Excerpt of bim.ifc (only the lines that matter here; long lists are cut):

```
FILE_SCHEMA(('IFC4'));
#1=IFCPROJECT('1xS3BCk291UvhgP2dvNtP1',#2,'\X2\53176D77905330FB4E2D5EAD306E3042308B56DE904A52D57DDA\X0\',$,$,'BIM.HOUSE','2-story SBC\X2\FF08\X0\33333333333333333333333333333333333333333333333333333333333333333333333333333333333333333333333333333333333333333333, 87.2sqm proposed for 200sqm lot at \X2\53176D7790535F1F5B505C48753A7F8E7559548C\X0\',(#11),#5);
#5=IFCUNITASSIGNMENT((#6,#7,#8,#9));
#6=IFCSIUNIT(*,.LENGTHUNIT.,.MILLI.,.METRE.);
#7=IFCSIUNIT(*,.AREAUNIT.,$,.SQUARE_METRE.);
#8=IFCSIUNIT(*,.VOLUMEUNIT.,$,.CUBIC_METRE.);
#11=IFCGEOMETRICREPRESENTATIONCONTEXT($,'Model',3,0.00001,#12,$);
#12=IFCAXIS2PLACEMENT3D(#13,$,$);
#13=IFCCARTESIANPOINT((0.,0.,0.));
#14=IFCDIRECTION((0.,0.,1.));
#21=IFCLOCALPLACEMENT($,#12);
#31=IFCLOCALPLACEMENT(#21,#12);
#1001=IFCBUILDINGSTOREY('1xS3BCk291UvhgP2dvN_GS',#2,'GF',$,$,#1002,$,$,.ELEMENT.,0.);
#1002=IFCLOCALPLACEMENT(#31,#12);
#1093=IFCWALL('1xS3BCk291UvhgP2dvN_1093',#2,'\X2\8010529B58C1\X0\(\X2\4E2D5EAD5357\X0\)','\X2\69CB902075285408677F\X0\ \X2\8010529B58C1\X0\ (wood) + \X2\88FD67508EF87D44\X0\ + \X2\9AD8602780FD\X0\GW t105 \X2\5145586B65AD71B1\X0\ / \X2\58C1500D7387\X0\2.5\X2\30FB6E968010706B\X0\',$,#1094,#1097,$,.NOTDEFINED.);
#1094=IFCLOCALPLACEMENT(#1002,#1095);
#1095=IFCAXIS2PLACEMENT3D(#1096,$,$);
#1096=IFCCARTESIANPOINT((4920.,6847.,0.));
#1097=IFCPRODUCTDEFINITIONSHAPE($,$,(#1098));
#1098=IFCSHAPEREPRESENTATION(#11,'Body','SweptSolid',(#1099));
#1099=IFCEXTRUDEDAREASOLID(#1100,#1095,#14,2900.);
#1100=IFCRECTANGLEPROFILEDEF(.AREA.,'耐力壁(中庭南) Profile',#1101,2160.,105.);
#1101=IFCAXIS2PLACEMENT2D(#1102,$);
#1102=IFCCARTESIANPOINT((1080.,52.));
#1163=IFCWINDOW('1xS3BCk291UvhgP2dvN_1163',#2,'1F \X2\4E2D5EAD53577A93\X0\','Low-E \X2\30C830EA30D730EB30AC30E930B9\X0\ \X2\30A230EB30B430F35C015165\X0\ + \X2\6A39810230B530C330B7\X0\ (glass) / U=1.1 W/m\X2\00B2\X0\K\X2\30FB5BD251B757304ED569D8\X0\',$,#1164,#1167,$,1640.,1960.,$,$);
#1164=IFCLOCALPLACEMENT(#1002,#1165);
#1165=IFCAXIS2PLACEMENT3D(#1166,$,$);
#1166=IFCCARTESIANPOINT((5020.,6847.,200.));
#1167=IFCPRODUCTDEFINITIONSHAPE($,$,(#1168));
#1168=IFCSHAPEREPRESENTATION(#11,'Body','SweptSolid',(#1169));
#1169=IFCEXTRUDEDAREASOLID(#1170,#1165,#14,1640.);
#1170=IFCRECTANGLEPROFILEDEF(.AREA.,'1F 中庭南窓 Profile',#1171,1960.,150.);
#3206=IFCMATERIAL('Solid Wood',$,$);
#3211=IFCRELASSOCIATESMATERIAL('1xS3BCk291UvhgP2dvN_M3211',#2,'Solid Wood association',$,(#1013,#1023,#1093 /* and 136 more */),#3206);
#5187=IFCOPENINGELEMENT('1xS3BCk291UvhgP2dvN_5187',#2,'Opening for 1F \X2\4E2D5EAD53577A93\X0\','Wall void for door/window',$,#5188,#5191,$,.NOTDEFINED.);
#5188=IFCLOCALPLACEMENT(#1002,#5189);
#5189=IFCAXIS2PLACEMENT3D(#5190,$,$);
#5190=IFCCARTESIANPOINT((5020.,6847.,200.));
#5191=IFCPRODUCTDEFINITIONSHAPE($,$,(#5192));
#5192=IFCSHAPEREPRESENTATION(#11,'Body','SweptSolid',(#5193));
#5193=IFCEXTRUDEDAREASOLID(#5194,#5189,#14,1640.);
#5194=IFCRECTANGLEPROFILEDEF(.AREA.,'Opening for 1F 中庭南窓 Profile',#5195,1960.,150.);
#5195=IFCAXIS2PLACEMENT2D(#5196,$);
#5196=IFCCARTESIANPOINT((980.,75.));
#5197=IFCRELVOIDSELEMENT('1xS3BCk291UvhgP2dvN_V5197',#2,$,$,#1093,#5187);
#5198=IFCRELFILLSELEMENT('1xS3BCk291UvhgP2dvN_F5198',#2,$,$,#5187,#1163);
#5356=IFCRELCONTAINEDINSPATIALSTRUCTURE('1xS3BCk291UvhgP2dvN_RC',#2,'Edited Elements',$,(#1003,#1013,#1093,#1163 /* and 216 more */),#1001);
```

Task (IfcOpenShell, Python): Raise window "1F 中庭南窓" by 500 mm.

```python
import numpy as np
import ifcopenshell
import ifcopenshell.api.geometry
import ifcopenshell.util.placement
import ifcopenshell.util.unit

model = ifcopenshell.open("bim.ifc")
unit_scale = ifcopenshell.util.unit.calculate_unit_scale(model)

window = model.by_guid("1xS3BCk291UvhgP2dvN_1163")
opening = window.FillsVoids[0].RelatingOpeningElement
dz = 500.0

shift = np.array([0.0, 0.0, dz])
# The window is not placed relative to its opening, so move both.
for product in (opening, window):
    matrix = ifcopenshell.util.placement.get_local_placement(product.ObjectPlacement)
    matrix[:3, 3] += shift
    ifcopenshell.api.geometry.edit_object_placement(model, product=product, matrix=matrix, is_si=False)

print(f"moved by {dz * unit_scale:+.3f} m")

model.write("bim_rev.ifc")
```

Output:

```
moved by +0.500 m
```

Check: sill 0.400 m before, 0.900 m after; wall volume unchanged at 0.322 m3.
